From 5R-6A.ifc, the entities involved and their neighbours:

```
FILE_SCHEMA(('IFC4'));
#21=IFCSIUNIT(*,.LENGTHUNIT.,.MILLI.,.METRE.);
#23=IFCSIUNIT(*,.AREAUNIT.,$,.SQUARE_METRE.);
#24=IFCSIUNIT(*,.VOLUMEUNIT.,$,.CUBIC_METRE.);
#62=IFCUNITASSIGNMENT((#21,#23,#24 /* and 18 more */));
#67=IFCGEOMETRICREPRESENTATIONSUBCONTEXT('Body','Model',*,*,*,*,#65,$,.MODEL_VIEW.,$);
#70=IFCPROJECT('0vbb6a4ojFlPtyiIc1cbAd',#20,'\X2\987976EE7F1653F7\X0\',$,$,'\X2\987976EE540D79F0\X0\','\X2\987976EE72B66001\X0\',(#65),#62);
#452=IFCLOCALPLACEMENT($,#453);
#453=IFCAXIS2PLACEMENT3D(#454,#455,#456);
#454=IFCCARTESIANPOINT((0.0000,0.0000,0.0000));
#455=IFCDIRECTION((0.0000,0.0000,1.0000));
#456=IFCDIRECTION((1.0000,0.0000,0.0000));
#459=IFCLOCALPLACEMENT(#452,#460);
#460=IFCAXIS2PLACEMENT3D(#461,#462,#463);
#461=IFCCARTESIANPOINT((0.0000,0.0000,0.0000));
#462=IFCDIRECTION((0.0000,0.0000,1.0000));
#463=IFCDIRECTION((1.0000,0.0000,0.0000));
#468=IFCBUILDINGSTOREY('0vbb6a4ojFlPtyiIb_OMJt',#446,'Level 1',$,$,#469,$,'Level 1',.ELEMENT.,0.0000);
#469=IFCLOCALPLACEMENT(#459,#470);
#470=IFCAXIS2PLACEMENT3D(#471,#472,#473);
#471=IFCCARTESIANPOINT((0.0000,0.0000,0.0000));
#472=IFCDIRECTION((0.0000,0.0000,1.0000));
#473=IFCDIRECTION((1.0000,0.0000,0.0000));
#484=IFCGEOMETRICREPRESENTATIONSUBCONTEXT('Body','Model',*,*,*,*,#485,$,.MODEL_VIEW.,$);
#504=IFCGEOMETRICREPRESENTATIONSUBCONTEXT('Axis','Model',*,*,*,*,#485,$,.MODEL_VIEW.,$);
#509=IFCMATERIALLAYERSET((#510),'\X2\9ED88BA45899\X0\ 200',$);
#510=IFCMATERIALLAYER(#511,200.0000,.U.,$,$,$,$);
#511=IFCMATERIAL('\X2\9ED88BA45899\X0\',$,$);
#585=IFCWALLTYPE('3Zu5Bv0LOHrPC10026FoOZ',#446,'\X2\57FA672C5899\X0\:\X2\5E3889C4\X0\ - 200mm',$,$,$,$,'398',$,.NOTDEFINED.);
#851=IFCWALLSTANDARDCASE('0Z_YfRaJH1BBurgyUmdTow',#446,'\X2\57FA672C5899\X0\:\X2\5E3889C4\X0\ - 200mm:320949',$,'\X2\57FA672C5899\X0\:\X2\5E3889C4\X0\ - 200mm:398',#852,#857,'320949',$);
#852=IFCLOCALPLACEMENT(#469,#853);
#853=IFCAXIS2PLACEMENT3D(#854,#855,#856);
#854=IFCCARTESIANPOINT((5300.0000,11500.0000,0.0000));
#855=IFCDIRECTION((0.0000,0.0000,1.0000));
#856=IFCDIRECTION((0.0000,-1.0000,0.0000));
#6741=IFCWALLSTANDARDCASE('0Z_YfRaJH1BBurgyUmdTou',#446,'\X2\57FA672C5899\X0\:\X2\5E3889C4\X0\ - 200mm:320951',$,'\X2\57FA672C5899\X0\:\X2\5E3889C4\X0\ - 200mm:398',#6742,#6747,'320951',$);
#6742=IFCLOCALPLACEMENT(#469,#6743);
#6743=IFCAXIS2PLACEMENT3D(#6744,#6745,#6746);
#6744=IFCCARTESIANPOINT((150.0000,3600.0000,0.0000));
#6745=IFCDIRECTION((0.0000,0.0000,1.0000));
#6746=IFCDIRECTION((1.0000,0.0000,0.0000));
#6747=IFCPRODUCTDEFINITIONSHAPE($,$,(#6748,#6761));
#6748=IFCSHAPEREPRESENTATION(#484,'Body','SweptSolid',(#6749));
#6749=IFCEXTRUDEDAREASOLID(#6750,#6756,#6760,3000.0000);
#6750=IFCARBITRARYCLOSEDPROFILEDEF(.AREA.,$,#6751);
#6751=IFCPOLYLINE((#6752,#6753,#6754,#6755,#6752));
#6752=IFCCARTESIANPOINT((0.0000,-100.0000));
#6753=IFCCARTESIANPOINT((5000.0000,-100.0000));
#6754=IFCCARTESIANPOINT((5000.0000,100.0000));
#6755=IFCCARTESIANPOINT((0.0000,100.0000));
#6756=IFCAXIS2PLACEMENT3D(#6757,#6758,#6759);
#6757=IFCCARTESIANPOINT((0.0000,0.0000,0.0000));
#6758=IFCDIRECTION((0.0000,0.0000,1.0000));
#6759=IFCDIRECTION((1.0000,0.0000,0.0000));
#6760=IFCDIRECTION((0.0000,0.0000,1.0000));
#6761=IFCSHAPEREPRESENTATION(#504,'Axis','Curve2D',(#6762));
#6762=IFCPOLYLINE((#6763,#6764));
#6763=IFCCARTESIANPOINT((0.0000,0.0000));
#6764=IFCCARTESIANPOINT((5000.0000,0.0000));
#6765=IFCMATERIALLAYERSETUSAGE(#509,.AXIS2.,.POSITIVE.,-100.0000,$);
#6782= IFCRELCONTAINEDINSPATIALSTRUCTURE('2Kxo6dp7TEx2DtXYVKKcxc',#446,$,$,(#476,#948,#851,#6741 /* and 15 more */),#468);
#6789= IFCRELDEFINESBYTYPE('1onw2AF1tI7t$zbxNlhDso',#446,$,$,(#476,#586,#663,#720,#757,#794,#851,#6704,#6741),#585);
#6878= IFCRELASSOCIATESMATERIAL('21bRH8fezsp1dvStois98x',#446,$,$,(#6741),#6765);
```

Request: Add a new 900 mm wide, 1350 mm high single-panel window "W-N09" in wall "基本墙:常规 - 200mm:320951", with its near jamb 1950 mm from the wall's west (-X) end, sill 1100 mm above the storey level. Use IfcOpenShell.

```python
import numpy as np
import ifcopenshell
import ifcopenshell.api.feature
import ifcopenshell.api.geometry
import ifcopenshell.api.root
import ifcopenshell.api.spatial
import ifcopenshell.geom
import ifcopenshell.util.element
import ifcopenshell.util.placement
import ifcopenshell.util.representation
import ifcopenshell.util.shape
import ifcopenshell.util.unit

model = ifcopenshell.open("5R-6A.ifc")
unit_scale = ifcopenshell.util.unit.calculate_unit_scale(model)
settings = ifcopenshell.geom.settings()


def volume(element):
    """Net volume in cubic metres, openings subtracted."""
    shape = ifcopenshell.geom.create_shape(settings, element)
    return ifcopenshell.util.shape.get_volume(shape.geometry)


wall = model.by_guid("0Z_YfRaJH1BBurgyUmdTou")
storey = ifcopenshell.util.element.get_container(wall, ifc_class="IfcBuildingStorey")
context = ifcopenshell.util.representation.get_context(model, "Model", "Body", "MODEL_VIEW")
before = volume(wall)

width, height, from_end, sill = 0.9, 1.35, 1.95, 1.1  # metres

# The wall runs along its own X axis, and the end named is its -X end.
wall_shape = ifcopenshell.geom.create_shape(settings, wall)
x, y, z = ifcopenshell.util.shape.get_vertices(wall_shape.geometry).T
start = x.min() + from_end
face, thickness = float(y.min()), float(y.max() - y.min())
wall_matrix = ifcopenshell.util.placement.get_local_placement(wall.ObjectPlacement)
level = ifcopenshell.util.placement.get_local_placement(storey.ObjectPlacement)[2, 3]


def in_wall(x, y):
    """Placement at x, y metres in the wall's axes, at sill height."""
    matrix = wall_matrix.copy()
    matrix[:, 3] = wall_matrix @ np.array([x / unit_scale, y / unit_scale, 0.0, 1.0])
    matrix[2, 3] = level + sill / unit_scale
    return matrix


# Opening: a box that overshoots both wall faces by 50 mm.
opening = ifcopenshell.api.root.create_entity(model, ifc_class="IfcOpeningElement", predefined_type="OPENING")
box = ifcopenshell.api.geometry.add_wall_representation(
    model, context=context, length=width, height=height, thickness=thickness + 0.1
)
ifcopenshell.api.geometry.assign_representation(model, product=opening, representation=box)
ifcopenshell.api.geometry.edit_object_placement(model, product=opening, matrix=in_wall(start, face - 0.05), is_si=False)
ifcopenshell.api.feature.add_feature(model, feature=opening, element=wall)

window = ifcopenshell.api.root.create_entity(model, ifc_class="IfcWindow", name="W-N09", predefined_type="WINDOW")
window.OverallWidth, window.OverallHeight = width / unit_scale, height / unit_scale
window.PartitioningType = "SINGLE_PANEL"
body = ifcopenshell.api.geometry.add_window_representation(
    model,
    context=context,
    overall_width=window.OverallWidth,
    overall_height=window.OverallHeight,
    partition_type="SINGLE_PANEL",
)
ifcopenshell.api.geometry.assign_representation(model, product=window, representation=body)
ifcopenshell.api.spatial.assign_container(model, products=[window], relating_structure=storey)
ifcopenshell.api.feature.add_filling(model, opening=opening, element=window)

# Centre the window in the wall's thickness.
ifcopenshell.api.geometry.edit_object_placement(model, product=window, matrix=in_wall(start, face), is_si=False)
window_shape = ifcopenshell.geom.create_shape(settings, window)
depth = ifcopenshell.util.shape.get_vertices(window_shape.geometry)[:, 1]
offset = face + thickness / 2 - (depth.min() + depth.max()) / 2
ifcopenshell.api.geometry.edit_object_placement(model, product=window, matrix=in_wall(start, offset), is_si=False)

after = volume(wall)

print(f"wall volume {before:.3f} -> {after:.3f} m3")

model.write("5R-6A_updated.ifc")
```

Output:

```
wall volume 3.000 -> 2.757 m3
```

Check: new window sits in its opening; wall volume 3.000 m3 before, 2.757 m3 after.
